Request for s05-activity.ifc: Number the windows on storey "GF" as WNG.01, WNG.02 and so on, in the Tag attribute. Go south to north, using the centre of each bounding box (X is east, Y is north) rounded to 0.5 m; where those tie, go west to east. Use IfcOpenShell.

First a look at what the model holds.

```python
import ifcopenshell
import ifcopenshell.util.element
import ifcopenshell.util.placement

model = ifcopenshell.open("s05-activity.ifc")
print(model.schema)
storey = next(s for s in model.by_type("IfcBuildingStorey") if s.Name == "GF")
windows = [e for e in ifcopenshell.util.element.get_decomposition(storey) if e.is_a("IfcWindow")]
for e in sorted(windows, key=lambda e: e.id()):
    origin = ifcopenshell.util.placement.get_local_placement(e.ObjectPlacement)[:3, 3]
    print(e.id(), e.Tag, e.Name, origin.round(2) + 0.0, sep=" | ")
```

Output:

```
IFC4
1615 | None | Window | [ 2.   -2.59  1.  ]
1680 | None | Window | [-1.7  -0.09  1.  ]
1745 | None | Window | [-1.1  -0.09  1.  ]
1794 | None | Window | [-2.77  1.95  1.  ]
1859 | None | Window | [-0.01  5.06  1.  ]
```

```python
import ifcopenshell
import ifcopenshell.geom
import ifcopenshell.util.element
import ifcopenshell.util.shape

model = ifcopenshell.open("s05-activity.ifc")
settings = ifcopenshell.geom.settings()
settings.set("use-world-coords", True)


def centre(element):
    shape = ifcopenshell.geom.create_shape(settings, element)
    return ifcopenshell.util.shape.get_bbox_centroid(shape.geometry)


storey = next(s for s in model.by_type("IfcBuildingStorey") if s.Name == "GF")
windows = [e for e in ifcopenshell.util.element.get_decomposition(storey) if e.is_a("IfcWindow")]

# Insertion points can sit at a corner or the storey origin, so sort by the geometry (in metres).
centres = {e: centre(e) for e in windows}
windows.sort(key=lambda e: (round(centres[e][1] / 0.5), centres[e][0]))

for i, e in enumerate(windows, start=1):
    number = f"WNG.{i:02d}"
    e.Tag = number
    print(e.id(), number)

model.write("s05-activity_v2.ifc")
```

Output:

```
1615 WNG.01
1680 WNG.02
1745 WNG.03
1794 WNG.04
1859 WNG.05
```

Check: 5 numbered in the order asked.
